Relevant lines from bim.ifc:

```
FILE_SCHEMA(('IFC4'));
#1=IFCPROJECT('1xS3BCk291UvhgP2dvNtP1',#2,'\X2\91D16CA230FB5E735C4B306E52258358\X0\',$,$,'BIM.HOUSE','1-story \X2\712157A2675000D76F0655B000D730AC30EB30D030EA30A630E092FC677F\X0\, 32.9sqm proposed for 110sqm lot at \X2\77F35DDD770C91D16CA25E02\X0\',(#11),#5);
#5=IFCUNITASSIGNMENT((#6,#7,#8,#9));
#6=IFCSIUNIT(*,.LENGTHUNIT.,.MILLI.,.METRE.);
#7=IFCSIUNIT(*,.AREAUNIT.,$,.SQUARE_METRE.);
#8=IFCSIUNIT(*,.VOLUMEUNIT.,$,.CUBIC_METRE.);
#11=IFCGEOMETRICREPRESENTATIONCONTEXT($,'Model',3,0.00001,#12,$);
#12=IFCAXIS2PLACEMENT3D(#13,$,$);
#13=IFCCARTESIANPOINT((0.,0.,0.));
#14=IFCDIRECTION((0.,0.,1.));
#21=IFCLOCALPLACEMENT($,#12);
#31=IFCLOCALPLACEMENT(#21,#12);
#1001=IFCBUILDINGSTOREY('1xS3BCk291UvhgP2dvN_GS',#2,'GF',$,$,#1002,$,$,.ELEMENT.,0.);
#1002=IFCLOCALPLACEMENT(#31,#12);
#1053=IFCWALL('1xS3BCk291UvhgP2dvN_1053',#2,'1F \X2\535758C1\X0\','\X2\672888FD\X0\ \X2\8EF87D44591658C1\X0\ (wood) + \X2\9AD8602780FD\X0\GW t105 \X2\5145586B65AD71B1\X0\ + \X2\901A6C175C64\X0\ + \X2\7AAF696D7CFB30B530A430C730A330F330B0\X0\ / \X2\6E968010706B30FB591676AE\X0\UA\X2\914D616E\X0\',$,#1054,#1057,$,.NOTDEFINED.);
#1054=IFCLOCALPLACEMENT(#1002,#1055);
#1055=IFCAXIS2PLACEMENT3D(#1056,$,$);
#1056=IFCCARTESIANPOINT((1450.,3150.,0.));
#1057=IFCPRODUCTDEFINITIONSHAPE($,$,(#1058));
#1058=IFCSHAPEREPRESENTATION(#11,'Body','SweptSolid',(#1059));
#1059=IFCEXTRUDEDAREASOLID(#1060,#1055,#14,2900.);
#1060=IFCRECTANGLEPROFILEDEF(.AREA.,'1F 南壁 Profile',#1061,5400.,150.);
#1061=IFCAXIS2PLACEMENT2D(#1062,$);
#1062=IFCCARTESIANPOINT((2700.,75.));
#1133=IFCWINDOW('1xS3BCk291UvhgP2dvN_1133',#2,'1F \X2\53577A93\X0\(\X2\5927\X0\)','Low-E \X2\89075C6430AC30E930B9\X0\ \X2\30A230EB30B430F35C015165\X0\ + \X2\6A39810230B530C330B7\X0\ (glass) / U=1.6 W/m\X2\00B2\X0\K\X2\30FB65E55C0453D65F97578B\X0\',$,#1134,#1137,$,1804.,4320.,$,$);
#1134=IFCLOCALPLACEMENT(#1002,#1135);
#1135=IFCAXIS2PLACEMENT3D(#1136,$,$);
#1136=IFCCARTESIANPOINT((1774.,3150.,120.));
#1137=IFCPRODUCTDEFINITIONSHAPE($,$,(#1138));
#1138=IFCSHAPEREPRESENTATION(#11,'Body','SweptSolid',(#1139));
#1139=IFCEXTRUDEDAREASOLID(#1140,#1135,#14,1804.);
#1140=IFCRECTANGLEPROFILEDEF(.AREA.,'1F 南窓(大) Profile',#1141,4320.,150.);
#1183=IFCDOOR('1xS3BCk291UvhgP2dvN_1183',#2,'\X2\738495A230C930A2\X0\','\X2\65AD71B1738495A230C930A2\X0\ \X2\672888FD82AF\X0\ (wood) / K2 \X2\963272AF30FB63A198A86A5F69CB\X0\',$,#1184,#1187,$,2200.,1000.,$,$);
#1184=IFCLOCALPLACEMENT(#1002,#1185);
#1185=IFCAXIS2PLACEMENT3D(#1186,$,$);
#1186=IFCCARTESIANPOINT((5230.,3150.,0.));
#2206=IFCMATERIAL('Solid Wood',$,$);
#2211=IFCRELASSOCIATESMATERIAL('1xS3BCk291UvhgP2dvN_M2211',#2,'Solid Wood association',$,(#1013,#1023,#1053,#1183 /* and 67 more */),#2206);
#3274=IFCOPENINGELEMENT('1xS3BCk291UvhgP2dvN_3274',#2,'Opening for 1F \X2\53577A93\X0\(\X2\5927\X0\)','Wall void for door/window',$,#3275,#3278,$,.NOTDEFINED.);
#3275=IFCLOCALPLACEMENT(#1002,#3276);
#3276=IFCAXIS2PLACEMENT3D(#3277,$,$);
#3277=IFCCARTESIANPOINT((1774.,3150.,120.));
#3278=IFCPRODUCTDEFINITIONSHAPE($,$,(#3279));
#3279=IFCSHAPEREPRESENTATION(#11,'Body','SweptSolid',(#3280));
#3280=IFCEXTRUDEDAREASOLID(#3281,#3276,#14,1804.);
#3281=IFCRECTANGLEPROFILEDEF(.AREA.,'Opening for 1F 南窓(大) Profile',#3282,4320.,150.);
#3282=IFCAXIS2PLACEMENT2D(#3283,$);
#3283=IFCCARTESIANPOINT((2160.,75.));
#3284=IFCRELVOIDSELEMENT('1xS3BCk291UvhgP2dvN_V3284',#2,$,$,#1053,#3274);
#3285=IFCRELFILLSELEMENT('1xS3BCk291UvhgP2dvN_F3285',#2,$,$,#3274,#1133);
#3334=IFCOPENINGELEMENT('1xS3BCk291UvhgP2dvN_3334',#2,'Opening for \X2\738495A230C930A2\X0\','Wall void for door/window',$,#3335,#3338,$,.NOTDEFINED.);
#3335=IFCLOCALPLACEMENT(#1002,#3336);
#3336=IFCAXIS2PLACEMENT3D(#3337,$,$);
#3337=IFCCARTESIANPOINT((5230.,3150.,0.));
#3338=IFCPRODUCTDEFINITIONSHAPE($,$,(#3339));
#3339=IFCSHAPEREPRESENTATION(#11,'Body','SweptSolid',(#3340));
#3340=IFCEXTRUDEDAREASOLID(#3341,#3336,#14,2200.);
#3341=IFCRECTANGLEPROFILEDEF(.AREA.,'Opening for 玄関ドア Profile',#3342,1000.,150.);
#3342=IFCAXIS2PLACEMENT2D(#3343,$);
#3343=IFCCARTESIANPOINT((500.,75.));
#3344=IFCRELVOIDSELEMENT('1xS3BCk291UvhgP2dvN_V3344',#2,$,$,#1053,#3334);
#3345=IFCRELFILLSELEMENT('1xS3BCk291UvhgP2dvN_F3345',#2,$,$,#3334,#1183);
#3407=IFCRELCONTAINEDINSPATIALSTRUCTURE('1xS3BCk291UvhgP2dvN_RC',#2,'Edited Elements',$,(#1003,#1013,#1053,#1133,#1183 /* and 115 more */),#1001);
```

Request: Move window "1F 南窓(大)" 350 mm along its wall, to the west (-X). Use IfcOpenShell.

```python
import ifcopenshell
import ifcopenshell.api.geometry
import ifcopenshell.util.placement

model = ifcopenshell.open("bim.ifc")

window = model.by_id(1133)
opening = window.FillsVoids[0].RelatingOpeningElement
wall = opening.VoidsElements[0].RelatingBuildingElement

wall_matrix = ifcopenshell.util.placement.get_local_placement(wall.ObjectPlacement)
shift = wall_matrix[:3, 0] * -350.0
before = ifcopenshell.util.placement.get_local_placement(window.ObjectPlacement)[:3, 3].copy()

# The window is not placed relative to its opening, so move both.
for product in (opening, window):
    matrix = ifcopenshell.util.placement.get_local_placement(product.ObjectPlacement)
    matrix[:3, 3] += shift
    ifcopenshell.api.geometry.edit_object_placement(model, product=product, matrix=matrix, is_si=False)

after = ifcopenshell.util.placement.get_local_placement(window.ObjectPlacement)[:3, 3]
print("window moved by", (after - before).round(3) + 0.0)

model.write("bim_rev.ifc")
```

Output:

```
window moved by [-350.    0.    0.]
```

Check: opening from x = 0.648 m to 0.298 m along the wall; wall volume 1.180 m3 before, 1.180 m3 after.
